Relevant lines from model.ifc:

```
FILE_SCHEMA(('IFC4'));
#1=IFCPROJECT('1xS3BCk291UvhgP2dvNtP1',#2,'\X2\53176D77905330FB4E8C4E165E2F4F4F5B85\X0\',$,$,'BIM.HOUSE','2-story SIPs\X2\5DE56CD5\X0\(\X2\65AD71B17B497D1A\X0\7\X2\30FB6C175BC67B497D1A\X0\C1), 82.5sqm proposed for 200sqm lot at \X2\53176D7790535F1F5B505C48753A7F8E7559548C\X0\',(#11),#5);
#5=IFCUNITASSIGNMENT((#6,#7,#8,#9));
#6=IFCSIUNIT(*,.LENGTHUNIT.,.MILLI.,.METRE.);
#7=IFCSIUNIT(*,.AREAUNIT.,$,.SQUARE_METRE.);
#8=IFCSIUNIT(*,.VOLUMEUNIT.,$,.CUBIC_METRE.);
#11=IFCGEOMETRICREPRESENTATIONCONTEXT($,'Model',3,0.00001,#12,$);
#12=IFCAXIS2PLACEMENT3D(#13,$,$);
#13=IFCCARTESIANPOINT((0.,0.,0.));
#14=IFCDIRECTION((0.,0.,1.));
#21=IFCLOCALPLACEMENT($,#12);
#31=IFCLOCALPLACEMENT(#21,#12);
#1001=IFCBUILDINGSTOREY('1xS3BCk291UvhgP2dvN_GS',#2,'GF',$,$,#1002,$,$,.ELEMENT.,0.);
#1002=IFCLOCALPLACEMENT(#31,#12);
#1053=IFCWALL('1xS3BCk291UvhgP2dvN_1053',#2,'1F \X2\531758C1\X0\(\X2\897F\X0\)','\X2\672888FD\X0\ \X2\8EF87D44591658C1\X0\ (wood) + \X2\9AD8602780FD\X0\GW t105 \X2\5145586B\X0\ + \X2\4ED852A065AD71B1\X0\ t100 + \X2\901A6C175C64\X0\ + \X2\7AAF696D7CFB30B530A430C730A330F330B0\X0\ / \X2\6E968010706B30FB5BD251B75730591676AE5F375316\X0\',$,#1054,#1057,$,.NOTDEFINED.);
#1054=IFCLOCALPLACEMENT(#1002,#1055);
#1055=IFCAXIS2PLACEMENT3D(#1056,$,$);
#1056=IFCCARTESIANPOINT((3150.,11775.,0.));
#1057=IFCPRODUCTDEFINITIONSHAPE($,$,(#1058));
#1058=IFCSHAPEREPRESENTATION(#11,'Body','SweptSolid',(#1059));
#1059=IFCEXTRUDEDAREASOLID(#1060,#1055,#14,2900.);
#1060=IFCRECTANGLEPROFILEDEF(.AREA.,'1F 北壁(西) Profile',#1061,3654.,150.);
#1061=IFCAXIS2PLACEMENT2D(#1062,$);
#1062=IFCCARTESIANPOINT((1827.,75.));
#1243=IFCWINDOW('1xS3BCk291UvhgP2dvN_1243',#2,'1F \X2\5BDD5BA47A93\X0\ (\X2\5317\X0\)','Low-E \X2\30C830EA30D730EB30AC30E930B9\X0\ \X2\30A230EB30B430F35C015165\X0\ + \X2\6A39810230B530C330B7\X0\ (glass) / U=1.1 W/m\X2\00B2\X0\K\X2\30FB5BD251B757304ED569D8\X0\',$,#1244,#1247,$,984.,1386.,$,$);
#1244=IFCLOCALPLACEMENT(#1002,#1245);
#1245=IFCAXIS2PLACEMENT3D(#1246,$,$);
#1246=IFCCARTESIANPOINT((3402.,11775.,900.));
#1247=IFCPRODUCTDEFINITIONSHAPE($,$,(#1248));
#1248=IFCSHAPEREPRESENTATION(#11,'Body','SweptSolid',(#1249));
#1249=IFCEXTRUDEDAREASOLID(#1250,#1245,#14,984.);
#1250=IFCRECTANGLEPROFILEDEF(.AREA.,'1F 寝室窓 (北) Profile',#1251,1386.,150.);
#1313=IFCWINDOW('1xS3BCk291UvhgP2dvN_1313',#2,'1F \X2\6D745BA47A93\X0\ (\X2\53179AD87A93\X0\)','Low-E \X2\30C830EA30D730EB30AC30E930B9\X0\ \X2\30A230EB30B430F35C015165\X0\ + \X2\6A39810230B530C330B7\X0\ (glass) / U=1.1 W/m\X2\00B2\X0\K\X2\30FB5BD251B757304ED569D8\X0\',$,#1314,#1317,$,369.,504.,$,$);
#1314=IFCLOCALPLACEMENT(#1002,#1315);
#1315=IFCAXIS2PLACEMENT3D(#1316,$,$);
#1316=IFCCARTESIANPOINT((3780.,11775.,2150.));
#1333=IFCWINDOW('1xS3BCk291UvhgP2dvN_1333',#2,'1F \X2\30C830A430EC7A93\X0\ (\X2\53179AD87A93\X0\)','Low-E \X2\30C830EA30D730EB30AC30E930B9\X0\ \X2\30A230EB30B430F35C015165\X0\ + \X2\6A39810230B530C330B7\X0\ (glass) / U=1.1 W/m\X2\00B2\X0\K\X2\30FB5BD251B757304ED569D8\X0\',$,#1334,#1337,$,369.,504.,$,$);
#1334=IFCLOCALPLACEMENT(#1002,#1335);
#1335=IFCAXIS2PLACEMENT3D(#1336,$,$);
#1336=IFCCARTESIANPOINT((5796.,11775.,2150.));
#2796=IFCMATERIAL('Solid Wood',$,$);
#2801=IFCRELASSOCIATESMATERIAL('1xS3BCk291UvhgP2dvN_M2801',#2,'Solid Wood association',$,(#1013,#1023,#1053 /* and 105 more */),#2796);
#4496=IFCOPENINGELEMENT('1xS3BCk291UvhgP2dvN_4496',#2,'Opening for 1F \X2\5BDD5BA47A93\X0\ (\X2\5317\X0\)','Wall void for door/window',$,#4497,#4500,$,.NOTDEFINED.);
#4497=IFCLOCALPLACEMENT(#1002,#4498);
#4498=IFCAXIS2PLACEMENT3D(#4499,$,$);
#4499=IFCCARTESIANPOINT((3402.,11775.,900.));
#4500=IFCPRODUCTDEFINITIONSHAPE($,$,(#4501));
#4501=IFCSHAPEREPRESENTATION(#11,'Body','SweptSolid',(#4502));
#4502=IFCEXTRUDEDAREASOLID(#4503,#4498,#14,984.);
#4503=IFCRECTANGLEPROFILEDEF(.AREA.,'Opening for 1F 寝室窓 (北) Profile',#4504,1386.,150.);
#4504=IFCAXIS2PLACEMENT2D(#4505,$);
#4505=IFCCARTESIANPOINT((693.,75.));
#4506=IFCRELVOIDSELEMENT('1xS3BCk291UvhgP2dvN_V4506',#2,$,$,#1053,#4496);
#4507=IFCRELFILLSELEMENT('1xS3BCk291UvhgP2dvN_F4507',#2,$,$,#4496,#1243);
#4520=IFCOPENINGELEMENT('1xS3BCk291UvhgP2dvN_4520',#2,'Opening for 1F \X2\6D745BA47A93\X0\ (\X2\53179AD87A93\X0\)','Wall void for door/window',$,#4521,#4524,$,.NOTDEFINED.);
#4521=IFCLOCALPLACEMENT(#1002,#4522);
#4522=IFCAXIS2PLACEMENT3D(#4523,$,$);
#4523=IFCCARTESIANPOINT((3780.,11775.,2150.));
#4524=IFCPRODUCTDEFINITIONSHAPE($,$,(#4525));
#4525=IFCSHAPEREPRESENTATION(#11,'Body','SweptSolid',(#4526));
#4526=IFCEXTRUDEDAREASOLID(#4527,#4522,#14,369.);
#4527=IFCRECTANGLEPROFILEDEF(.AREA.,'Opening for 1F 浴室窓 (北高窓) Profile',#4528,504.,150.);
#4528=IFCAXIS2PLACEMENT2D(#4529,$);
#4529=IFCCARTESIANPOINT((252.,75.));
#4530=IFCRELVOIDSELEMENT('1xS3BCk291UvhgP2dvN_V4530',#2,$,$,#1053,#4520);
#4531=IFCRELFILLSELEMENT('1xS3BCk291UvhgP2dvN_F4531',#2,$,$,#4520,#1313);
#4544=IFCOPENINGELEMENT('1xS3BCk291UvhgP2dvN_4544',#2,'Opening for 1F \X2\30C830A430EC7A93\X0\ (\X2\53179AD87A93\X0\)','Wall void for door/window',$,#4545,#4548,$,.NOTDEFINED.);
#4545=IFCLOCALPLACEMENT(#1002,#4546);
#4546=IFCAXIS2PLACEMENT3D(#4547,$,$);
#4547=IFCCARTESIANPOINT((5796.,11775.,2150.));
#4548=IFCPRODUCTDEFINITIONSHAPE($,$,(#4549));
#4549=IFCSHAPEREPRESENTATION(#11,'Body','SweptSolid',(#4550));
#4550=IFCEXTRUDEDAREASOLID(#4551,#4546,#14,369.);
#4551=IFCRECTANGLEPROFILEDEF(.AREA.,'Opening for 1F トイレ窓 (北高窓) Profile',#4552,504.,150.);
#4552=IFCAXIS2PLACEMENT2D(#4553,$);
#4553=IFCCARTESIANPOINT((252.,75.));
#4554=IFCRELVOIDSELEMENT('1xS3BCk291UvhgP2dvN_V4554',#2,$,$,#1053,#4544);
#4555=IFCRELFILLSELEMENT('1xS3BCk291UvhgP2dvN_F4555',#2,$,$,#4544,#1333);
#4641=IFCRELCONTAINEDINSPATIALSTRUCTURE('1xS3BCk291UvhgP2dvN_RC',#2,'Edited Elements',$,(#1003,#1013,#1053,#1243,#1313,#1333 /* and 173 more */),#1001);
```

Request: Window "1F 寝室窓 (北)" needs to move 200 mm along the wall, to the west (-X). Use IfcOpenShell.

```python
import ifcopenshell
import ifcopenshell.api.geometry
import ifcopenshell.util.placement
import ifcopenshell.util.unit

model = ifcopenshell.open("model.ifc")
unit_scale = ifcopenshell.util.unit.calculate_unit_scale(model)

window = model.by_guid("1xS3BCk291UvhgP2dvN_1243")
opening = window.FillsVoids[0].RelatingOpeningElement
wall = opening.VoidsElements[0].RelatingBuildingElement

wall_matrix = ifcopenshell.util.placement.get_local_placement(wall.ObjectPlacement)
shift = wall_matrix[:3, 0] * -0.2 / unit_scale
before = ifcopenshell.util.placement.get_local_placement(window.ObjectPlacement)[:3, 3].copy()

# The window is not placed relative to its opening, so move both.
for product in (opening, window):
    matrix = ifcopenshell.util.placement.get_local_placement(product.ObjectPlacement)
    matrix[:3, 3] += shift
    ifcopenshell.api.geometry.edit_object_placement(model, product=product, matrix=matrix, is_si=False)

after = ifcopenshell.util.placement.get_local_placement(window.ObjectPlacement)[:3, 3]
print("window moved by", (after - before).round(3) + 0.0)

model.write("model_v2.ifc")
```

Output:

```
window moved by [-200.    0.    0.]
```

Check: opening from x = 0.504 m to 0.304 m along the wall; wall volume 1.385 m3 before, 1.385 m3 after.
